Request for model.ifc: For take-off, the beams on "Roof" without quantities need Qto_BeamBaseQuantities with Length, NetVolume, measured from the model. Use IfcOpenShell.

First a look at what the model holds.

```python
import ifcopenshell
import ifcopenshell.util.element
import ifcopenshell.util.unit

model = ifcopenshell.open("model.ifc")
print(model.schema)
for unit_type in ("LENGTHUNIT", "AREAUNIT", "VOLUMEUNIT"):
    print(unit_type, ifcopenshell.util.unit.calculate_unit_scale(model, unit_type))
storey = next(s for s in model.by_type("IfcBuildingStorey") if s.Name == "Roof")
beams = [e for e in ifcopenshell.util.element.get_decomposition(storey) if e.is_a("IfcBeam")]
for e in sorted(beams, key=lambda e: e.id()):
    print(e.id(), e.is_a(), e.Name, list(ifcopenshell.util.element.get_psets(e, qtos_only=True)), sep=" | ")
```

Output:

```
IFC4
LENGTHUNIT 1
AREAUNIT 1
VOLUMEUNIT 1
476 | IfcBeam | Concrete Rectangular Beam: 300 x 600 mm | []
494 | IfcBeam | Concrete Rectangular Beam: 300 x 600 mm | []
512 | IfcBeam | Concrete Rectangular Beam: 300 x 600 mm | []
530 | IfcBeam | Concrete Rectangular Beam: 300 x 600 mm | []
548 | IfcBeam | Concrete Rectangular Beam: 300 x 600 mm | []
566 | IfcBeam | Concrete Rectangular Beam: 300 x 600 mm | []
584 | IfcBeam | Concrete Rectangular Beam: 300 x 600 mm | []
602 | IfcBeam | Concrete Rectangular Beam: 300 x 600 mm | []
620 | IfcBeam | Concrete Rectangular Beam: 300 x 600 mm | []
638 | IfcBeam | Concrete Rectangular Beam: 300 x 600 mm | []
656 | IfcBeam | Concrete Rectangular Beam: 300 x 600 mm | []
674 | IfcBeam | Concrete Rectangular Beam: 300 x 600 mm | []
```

```python
import ifcopenshell
import ifcopenshell.api.pset
import ifcopenshell.geom
import ifcopenshell.util.element
import ifcopenshell.util.shape
import ifcopenshell.util.unit

model = ifcopenshell.open("model.ifc")
unit_scale = ifcopenshell.util.unit.calculate_unit_scale(model)
volume_scale = ifcopenshell.util.unit.calculate_unit_scale(model, "VOLUMEUNIT")
settings = ifcopenshell.geom.settings()

storey = next(s for s in model.by_type("IfcBuildingStorey") if s.Name == "Roof")
beams = [e for e in ifcopenshell.util.element.get_decomposition(storey) if e.is_a("IfcBeam")]

for e in sorted(beams, key=lambda e: e.id()):
    if ifcopenshell.util.element.get_psets(e, qtos_only=True, should_inherit=False):
        continue
    # Geometry comes back in metres, in the element's own axes.
    shape = ifcopenshell.geom.create_shape(settings, e)
    values = {
        "Length": ifcopenshell.util.shape.get_max_xyz(shape.geometry) / unit_scale,
        "NetVolume": ifcopenshell.util.shape.get_volume(shape.geometry) / volume_scale,
    }
    qto = ifcopenshell.api.pset.add_qto(model, product=e, name="Qto_BeamBaseQuantities")
    ifcopenshell.api.pset.edit_qto(model, qto=qto, properties=values)
    print(e.id(), {k: round(v, 3) for k, v in values.items()})

model.write("model_edited.ifc")
```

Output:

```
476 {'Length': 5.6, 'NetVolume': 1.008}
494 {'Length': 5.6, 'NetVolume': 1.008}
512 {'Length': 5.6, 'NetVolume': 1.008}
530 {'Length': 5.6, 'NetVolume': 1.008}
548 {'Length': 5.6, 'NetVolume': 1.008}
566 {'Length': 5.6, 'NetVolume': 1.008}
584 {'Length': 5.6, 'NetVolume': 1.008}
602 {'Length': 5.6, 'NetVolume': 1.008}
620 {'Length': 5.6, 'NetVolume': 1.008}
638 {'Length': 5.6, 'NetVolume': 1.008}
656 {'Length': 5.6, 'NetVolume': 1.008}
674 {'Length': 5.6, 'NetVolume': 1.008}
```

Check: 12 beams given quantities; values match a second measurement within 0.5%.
